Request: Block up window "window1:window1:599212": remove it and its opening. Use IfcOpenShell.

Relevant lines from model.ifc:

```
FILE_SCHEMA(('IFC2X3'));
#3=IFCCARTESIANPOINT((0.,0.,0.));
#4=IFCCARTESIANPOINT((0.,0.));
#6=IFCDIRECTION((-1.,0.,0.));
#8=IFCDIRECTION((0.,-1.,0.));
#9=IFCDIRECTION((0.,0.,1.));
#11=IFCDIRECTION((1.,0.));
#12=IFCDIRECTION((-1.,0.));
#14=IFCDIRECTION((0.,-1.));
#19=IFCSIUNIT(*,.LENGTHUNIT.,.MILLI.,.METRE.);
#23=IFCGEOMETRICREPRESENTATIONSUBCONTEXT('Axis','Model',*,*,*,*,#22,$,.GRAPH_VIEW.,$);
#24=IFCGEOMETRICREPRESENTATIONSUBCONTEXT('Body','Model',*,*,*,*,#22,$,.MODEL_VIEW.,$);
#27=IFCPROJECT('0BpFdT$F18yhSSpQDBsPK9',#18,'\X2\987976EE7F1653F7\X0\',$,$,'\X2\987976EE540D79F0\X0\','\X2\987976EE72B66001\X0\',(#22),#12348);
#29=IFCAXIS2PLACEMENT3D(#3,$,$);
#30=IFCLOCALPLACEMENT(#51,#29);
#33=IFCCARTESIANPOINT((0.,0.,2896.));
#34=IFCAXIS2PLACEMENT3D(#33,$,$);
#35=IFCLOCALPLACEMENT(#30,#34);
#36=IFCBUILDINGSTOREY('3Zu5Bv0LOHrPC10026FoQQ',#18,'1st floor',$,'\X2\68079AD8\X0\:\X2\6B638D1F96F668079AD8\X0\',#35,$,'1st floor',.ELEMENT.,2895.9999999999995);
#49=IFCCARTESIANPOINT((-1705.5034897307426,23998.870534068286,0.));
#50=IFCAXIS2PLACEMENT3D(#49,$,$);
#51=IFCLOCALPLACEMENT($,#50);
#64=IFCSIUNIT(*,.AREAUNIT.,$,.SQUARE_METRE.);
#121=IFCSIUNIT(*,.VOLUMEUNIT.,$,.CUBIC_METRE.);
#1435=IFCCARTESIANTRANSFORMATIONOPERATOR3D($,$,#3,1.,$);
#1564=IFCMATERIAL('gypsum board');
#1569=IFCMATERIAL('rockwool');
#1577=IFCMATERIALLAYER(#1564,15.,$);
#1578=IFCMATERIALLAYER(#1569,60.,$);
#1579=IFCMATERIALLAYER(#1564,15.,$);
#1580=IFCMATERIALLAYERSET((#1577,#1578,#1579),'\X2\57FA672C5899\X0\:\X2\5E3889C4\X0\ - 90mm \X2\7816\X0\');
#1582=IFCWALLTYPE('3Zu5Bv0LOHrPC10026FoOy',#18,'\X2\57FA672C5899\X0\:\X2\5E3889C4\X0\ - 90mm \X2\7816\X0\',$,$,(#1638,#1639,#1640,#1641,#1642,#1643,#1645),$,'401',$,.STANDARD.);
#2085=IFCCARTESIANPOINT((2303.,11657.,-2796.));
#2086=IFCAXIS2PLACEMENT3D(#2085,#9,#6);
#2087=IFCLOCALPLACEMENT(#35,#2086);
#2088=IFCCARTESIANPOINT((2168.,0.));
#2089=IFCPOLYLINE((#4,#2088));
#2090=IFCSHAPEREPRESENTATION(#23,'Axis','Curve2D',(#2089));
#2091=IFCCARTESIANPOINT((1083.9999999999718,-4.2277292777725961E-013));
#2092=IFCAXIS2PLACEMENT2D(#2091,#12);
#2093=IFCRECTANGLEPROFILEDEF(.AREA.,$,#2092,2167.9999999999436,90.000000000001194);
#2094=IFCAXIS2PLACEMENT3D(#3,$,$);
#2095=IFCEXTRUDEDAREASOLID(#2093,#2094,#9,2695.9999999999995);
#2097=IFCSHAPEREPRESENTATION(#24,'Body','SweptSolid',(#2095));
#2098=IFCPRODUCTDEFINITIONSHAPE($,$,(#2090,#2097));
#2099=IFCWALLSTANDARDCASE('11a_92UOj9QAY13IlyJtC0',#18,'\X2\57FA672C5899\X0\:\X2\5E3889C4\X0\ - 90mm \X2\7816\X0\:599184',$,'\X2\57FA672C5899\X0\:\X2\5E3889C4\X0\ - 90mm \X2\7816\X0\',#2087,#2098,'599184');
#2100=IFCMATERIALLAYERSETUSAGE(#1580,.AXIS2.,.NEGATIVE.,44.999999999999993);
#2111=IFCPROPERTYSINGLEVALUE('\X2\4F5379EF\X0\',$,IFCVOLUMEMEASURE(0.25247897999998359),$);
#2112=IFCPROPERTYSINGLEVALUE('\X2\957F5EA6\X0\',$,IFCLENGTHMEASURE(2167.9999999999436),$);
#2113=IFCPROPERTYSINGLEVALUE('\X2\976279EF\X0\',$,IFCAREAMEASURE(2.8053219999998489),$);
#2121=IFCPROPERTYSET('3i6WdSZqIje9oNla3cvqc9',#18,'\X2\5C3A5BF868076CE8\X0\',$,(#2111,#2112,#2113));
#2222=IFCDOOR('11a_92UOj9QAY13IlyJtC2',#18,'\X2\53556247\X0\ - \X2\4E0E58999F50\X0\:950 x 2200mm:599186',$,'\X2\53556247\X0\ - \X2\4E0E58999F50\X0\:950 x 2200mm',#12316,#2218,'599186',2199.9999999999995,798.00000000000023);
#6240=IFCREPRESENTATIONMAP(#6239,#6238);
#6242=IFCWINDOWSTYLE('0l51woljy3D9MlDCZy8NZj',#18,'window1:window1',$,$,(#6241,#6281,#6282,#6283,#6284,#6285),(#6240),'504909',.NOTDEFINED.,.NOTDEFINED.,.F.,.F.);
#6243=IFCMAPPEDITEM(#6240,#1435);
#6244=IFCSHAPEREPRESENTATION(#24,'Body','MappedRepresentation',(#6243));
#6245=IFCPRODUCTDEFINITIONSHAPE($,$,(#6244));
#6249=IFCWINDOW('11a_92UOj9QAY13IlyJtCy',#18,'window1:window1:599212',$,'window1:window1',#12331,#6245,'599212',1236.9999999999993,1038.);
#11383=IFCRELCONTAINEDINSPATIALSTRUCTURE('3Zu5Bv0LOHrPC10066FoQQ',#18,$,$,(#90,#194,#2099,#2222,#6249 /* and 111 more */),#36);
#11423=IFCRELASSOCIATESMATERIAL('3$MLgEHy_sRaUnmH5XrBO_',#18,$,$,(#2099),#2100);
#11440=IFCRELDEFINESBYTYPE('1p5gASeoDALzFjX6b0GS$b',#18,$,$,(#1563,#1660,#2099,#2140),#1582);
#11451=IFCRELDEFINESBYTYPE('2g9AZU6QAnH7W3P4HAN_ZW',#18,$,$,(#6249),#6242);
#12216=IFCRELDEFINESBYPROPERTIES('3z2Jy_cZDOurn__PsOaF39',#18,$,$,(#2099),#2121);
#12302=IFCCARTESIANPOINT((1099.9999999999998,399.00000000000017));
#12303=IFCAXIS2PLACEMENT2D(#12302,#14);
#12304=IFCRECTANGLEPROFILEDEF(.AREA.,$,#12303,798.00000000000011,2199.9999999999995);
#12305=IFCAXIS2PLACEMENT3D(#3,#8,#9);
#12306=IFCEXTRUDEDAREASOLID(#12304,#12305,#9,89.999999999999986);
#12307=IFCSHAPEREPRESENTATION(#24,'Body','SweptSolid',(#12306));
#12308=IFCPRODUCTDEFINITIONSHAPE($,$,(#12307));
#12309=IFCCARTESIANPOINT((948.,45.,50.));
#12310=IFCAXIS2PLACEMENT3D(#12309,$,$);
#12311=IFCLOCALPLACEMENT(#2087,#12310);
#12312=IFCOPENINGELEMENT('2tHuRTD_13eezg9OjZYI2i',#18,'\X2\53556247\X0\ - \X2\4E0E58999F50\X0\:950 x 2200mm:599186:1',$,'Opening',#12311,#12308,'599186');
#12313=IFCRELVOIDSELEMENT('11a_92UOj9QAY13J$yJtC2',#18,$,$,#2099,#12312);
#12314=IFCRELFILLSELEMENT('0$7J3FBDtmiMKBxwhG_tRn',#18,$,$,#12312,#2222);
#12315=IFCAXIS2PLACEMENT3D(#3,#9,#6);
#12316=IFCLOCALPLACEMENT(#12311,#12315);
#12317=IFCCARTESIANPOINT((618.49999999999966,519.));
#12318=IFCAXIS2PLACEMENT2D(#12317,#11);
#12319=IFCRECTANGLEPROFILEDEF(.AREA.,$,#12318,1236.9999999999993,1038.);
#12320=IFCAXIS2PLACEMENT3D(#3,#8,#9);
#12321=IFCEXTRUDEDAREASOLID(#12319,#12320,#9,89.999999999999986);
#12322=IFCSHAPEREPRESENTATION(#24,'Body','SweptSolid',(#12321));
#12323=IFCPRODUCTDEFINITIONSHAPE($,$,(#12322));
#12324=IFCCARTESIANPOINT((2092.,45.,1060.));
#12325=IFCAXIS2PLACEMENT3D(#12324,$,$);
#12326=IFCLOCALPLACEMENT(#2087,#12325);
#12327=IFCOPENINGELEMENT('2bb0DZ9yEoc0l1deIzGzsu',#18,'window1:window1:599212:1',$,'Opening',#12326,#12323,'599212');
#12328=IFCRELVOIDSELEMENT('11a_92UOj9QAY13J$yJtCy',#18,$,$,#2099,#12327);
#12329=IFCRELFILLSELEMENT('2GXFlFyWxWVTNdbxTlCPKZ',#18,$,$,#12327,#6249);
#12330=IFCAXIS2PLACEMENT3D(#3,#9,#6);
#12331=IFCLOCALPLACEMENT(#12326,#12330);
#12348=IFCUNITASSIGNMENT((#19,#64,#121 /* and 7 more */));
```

```python
import ifcopenshell
import ifcopenshell.api.feature
import ifcopenshell.api.pset
import ifcopenshell.api.root
import ifcopenshell.geom
import ifcopenshell.util.element
import ifcopenshell.util.shape
import ifcopenshell.util.unit

model = ifcopenshell.open("model.ifc")
area_scale = ifcopenshell.util.unit.calculate_unit_scale(model, "AREAUNIT")
volume_scale = ifcopenshell.util.unit.calculate_unit_scale(model, "VOLUMEUNIT")
settings = ifcopenshell.geom.settings()


def volume(element):
    """Net volume in cubic metres, openings subtracted."""
    shape = ifcopenshell.geom.create_shape(settings, element)
    return ifcopenshell.util.shape.get_volume(shape.geometry)


window = model.by_id(6249)
opening = window.FillsVoids[0].RelatingOpeningElement
wall = opening.VoidsElements[0].RelatingBuildingElement
before = volume(wall)

ifcopenshell.api.root.remove_product(model, product=window)
ifcopenshell.api.feature.remove_feature(model, feature=opening)

after = volume(wall)
thickness = 0.09  # wall thickness in metres

# Update the wall's stored quantities.
pset = model.by_id(ifcopenshell.util.element.get_pset(wall, "尺寸标注", should_inherit=False)["id"])
ifcopenshell.api.pset.edit_pset(model, pset=pset, properties={
    "体积": model.create_entity("IfcVolumeMeasure", after / volume_scale),
    "面积": model.create_entity("IfcAreaMeasure", after / thickness / area_scale),
})

print(f"wall volume {before:.3f} -> {after:.3f} m3")

model.write("model-out.ifc")
```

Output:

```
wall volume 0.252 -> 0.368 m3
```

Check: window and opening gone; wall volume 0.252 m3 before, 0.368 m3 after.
